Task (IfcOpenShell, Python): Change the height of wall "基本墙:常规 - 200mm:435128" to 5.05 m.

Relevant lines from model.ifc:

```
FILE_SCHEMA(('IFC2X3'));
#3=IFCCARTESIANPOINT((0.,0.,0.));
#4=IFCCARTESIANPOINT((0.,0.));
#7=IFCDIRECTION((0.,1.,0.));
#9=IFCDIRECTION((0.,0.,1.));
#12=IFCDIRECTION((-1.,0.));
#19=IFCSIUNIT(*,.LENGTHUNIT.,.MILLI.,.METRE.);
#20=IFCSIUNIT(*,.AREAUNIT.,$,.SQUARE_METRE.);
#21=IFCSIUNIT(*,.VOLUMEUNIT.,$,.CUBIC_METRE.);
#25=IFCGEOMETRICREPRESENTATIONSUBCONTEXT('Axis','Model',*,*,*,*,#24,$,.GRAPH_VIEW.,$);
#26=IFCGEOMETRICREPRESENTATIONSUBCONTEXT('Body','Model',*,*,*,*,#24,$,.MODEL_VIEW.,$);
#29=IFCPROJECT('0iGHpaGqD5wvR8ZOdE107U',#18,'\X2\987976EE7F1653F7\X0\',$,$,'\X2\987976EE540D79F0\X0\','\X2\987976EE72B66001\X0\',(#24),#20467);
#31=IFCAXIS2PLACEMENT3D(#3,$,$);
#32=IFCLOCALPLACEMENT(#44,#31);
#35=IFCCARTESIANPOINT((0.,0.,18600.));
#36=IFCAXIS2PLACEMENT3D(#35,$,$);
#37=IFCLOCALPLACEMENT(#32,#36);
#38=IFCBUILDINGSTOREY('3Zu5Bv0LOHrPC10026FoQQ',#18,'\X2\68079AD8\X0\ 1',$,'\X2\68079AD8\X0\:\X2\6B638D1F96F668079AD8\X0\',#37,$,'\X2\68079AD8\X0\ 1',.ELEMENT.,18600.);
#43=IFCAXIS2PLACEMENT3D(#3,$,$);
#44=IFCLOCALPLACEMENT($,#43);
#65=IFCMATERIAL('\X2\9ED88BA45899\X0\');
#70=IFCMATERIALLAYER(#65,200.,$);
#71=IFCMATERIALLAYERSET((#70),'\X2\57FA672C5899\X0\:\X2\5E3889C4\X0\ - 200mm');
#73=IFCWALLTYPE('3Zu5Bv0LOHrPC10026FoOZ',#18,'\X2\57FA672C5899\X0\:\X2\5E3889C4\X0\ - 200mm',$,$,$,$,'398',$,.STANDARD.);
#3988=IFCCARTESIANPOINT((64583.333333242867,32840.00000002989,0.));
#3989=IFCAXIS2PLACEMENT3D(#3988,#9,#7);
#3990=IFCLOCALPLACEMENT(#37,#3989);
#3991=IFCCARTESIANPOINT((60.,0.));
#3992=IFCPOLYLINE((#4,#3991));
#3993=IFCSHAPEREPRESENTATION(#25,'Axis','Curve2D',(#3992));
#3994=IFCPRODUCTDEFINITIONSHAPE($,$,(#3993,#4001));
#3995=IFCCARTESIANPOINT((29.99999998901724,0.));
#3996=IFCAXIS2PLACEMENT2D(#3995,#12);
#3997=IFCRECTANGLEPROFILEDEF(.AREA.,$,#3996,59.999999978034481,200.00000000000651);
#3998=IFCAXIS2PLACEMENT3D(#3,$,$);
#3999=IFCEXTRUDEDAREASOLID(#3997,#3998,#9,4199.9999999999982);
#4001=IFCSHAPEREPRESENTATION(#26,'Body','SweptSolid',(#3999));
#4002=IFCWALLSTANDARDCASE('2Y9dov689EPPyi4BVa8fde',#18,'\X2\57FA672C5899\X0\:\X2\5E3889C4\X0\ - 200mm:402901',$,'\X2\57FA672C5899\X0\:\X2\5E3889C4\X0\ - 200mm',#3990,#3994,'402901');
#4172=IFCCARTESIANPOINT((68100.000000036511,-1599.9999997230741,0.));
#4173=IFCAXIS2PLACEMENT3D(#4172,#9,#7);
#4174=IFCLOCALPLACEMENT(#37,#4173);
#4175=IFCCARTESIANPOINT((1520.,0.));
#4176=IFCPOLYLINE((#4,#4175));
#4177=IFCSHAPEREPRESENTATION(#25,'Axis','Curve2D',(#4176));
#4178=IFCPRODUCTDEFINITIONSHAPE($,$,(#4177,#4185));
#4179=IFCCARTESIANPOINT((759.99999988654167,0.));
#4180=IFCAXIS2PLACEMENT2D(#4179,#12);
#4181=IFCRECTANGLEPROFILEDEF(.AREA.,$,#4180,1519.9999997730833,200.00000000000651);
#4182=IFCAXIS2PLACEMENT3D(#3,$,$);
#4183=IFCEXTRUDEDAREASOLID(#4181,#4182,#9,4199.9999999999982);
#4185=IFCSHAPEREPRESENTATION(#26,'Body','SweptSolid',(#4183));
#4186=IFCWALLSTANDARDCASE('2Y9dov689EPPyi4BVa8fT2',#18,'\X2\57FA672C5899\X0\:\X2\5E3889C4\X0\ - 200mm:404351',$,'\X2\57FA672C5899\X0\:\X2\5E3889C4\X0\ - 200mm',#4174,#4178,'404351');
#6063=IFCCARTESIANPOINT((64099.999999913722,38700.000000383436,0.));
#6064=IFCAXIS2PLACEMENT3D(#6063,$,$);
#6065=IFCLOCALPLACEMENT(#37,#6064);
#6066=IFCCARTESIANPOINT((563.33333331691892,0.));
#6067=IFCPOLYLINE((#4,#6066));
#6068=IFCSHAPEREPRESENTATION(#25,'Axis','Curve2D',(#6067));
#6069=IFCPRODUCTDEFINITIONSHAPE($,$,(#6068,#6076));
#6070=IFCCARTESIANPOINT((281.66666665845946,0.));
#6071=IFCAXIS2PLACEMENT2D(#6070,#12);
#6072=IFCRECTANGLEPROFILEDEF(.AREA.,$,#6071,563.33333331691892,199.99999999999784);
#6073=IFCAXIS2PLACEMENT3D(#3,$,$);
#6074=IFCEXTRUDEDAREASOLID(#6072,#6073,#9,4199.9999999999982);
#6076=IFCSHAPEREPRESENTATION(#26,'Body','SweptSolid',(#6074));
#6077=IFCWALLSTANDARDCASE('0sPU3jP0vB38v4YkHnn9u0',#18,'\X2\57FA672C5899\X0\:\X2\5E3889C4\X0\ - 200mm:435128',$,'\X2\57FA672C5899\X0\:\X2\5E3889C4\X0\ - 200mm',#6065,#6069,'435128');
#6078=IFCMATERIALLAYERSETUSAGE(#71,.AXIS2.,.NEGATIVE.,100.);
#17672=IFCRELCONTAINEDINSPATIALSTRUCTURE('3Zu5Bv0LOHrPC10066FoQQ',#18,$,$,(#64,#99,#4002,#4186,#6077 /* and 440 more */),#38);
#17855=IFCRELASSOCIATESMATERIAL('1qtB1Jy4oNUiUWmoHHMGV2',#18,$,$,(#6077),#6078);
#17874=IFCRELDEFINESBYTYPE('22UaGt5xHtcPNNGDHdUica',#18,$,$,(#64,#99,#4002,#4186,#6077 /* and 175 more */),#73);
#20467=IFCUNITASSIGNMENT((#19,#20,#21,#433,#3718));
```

```python
import ifcopenshell
import ifcopenshell.geom
import ifcopenshell.util.representation
import ifcopenshell.util.shape
import ifcopenshell.util.unit

model = ifcopenshell.open("model.ifc")
unit_scale = ifcopenshell.util.unit.calculate_unit_scale(model)
settings = ifcopenshell.geom.settings()


def volume(element):
    """Net volume in cubic metres, openings subtracted."""
    shape = ifcopenshell.geom.create_shape(settings, element)
    return ifcopenshell.util.shape.get_volume(shape.geometry)


wall = model.by_guid("0sPU3jP0vB38v4YkHnn9u0")
before = volume(wall)

body = ifcopenshell.util.representation.get_representation(wall, "Model", "Body")
solid = body.Items[0]
old_height = solid.Depth
solid.Depth = 5.05 / unit_scale
after = volume(wall)

print(f"height {old_height:g} -> {solid.Depth:g}, volume {before:.3f} -> {after:.3f} m3")

model.write("model_v2.ifc")
```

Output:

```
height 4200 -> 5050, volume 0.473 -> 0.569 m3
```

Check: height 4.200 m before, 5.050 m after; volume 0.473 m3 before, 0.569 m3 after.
